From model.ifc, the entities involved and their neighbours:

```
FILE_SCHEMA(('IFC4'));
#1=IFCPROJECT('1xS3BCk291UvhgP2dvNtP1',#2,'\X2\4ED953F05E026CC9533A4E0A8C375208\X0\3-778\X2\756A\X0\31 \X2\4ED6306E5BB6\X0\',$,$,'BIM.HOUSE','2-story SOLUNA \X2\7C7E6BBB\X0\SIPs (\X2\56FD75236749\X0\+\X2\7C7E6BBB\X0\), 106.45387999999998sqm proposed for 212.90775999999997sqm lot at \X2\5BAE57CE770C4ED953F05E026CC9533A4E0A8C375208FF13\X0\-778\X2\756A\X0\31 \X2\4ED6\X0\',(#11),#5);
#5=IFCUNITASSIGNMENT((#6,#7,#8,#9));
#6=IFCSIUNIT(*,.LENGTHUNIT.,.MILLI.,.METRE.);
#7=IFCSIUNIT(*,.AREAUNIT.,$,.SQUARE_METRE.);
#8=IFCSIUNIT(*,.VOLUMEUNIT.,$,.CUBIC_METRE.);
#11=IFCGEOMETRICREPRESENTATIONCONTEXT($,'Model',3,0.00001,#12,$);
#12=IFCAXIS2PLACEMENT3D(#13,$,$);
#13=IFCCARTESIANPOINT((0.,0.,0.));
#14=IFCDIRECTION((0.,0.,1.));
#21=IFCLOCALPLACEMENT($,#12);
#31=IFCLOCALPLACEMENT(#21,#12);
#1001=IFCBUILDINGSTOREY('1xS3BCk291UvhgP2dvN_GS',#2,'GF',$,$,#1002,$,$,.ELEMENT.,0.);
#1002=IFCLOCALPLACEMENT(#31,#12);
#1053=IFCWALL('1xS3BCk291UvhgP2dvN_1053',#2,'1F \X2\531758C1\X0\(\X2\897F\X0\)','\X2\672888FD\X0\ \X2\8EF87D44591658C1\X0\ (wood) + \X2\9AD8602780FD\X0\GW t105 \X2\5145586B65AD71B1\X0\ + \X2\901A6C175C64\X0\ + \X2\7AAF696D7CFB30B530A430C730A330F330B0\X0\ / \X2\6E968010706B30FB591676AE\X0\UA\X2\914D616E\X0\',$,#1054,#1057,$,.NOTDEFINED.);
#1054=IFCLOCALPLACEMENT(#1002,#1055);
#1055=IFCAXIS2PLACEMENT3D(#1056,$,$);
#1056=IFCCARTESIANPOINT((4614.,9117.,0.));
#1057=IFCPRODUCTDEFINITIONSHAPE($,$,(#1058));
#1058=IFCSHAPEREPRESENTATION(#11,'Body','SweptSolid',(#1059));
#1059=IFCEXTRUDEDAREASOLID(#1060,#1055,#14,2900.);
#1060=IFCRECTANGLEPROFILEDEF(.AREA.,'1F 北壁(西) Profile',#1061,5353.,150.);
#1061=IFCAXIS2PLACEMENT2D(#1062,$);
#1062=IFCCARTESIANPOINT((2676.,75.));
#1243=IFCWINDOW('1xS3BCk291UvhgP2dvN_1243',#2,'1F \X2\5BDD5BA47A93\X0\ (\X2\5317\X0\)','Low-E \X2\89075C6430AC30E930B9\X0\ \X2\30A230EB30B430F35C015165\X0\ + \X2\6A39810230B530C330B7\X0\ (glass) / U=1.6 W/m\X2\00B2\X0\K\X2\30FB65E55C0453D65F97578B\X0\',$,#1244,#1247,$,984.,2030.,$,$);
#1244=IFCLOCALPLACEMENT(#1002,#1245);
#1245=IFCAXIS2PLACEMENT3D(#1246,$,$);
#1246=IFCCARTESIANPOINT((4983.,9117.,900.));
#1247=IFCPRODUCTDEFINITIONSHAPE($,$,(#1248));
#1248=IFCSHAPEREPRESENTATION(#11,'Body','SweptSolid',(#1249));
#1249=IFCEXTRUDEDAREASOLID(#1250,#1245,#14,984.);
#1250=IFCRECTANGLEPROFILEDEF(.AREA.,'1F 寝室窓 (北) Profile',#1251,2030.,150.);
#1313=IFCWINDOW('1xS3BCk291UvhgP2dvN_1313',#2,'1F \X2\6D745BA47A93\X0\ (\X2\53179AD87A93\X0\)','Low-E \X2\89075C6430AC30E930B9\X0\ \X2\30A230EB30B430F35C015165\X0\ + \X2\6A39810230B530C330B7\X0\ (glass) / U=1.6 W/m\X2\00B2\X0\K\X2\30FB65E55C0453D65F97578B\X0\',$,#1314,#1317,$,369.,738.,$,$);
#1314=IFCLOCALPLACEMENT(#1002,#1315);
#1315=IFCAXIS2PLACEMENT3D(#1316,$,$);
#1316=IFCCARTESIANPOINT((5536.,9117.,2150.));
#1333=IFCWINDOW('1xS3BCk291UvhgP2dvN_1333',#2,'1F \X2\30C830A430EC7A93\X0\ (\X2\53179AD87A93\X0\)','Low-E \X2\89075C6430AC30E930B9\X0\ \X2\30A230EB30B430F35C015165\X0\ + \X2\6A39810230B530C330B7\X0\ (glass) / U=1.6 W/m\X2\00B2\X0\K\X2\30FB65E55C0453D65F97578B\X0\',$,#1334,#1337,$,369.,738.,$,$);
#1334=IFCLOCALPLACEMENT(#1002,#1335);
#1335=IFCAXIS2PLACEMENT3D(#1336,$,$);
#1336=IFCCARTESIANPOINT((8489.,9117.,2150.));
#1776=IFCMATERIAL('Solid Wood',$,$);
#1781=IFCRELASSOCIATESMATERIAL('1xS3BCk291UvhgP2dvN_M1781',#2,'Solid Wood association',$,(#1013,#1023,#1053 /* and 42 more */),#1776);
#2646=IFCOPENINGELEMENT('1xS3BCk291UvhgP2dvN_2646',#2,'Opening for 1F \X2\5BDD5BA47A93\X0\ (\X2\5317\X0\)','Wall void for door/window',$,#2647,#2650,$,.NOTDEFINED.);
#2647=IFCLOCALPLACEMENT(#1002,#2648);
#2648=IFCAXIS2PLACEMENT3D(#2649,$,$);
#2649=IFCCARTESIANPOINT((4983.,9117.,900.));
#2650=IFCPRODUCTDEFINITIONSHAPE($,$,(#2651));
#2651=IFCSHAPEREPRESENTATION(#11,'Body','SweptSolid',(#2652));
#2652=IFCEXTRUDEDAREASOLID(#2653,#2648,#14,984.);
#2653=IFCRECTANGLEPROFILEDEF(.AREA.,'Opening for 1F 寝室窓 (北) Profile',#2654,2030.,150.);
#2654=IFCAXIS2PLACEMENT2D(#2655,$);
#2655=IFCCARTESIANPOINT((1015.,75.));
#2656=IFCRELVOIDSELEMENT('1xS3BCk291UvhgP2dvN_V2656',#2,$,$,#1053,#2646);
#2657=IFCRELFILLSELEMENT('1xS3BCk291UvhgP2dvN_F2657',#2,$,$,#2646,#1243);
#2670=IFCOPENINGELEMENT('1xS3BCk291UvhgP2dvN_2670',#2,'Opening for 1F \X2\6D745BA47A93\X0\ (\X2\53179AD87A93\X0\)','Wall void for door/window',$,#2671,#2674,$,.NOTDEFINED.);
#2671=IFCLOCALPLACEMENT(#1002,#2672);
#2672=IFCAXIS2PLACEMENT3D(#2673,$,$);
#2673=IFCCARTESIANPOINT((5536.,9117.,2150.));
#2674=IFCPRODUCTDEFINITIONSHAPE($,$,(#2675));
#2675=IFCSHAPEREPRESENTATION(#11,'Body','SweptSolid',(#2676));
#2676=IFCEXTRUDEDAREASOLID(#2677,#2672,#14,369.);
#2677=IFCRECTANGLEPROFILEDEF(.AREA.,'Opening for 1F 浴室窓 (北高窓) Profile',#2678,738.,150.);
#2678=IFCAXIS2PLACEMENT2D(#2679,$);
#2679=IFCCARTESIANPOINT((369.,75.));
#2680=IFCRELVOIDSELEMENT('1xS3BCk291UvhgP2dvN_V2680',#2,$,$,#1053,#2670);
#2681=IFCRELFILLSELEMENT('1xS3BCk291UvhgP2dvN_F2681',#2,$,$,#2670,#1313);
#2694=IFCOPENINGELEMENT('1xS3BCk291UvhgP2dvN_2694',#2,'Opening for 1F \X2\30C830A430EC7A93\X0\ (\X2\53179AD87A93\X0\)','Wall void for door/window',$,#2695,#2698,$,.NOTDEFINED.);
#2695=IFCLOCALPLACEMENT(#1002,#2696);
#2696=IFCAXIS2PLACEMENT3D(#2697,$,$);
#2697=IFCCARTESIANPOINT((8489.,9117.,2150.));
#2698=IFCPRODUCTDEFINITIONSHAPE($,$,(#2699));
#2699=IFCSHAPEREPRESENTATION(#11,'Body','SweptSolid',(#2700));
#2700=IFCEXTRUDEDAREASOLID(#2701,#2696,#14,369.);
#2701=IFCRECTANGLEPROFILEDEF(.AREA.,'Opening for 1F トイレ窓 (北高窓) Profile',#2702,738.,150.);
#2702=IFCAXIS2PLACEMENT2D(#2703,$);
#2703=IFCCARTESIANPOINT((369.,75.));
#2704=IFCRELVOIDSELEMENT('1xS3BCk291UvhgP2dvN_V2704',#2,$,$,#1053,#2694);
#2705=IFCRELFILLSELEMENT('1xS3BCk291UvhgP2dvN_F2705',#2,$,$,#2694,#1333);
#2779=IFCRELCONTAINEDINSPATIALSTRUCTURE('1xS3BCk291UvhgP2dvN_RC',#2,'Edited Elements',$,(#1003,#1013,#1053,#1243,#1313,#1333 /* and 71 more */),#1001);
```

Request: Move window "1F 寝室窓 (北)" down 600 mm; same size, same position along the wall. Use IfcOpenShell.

```python
import numpy as np
import ifcopenshell
import ifcopenshell.api.geometry
import ifcopenshell.util.placement
import ifcopenshell.util.unit

model = ifcopenshell.open("model.ifc")
unit_scale = ifcopenshell.util.unit.calculate_unit_scale(model)

window = model.by_guid("1xS3BCk291UvhgP2dvN_1243")
opening = window.FillsVoids[0].RelatingOpeningElement
dz = -0.6 / unit_scale

shift = np.array([0.0, 0.0, dz])
# The window is not placed relative to its opening, so move both.
for product in (opening, window):
    matrix = ifcopenshell.util.placement.get_local_placement(product.ObjectPlacement)
    matrix[:3, 3] += shift
    ifcopenshell.api.geometry.edit_object_placement(model, product=product, matrix=matrix, is_si=False)

print(f"moved by {dz * unit_scale:+.3f} m")

model.write("model_v2.ifc")
```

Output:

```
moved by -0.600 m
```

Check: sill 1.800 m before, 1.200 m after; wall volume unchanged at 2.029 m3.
